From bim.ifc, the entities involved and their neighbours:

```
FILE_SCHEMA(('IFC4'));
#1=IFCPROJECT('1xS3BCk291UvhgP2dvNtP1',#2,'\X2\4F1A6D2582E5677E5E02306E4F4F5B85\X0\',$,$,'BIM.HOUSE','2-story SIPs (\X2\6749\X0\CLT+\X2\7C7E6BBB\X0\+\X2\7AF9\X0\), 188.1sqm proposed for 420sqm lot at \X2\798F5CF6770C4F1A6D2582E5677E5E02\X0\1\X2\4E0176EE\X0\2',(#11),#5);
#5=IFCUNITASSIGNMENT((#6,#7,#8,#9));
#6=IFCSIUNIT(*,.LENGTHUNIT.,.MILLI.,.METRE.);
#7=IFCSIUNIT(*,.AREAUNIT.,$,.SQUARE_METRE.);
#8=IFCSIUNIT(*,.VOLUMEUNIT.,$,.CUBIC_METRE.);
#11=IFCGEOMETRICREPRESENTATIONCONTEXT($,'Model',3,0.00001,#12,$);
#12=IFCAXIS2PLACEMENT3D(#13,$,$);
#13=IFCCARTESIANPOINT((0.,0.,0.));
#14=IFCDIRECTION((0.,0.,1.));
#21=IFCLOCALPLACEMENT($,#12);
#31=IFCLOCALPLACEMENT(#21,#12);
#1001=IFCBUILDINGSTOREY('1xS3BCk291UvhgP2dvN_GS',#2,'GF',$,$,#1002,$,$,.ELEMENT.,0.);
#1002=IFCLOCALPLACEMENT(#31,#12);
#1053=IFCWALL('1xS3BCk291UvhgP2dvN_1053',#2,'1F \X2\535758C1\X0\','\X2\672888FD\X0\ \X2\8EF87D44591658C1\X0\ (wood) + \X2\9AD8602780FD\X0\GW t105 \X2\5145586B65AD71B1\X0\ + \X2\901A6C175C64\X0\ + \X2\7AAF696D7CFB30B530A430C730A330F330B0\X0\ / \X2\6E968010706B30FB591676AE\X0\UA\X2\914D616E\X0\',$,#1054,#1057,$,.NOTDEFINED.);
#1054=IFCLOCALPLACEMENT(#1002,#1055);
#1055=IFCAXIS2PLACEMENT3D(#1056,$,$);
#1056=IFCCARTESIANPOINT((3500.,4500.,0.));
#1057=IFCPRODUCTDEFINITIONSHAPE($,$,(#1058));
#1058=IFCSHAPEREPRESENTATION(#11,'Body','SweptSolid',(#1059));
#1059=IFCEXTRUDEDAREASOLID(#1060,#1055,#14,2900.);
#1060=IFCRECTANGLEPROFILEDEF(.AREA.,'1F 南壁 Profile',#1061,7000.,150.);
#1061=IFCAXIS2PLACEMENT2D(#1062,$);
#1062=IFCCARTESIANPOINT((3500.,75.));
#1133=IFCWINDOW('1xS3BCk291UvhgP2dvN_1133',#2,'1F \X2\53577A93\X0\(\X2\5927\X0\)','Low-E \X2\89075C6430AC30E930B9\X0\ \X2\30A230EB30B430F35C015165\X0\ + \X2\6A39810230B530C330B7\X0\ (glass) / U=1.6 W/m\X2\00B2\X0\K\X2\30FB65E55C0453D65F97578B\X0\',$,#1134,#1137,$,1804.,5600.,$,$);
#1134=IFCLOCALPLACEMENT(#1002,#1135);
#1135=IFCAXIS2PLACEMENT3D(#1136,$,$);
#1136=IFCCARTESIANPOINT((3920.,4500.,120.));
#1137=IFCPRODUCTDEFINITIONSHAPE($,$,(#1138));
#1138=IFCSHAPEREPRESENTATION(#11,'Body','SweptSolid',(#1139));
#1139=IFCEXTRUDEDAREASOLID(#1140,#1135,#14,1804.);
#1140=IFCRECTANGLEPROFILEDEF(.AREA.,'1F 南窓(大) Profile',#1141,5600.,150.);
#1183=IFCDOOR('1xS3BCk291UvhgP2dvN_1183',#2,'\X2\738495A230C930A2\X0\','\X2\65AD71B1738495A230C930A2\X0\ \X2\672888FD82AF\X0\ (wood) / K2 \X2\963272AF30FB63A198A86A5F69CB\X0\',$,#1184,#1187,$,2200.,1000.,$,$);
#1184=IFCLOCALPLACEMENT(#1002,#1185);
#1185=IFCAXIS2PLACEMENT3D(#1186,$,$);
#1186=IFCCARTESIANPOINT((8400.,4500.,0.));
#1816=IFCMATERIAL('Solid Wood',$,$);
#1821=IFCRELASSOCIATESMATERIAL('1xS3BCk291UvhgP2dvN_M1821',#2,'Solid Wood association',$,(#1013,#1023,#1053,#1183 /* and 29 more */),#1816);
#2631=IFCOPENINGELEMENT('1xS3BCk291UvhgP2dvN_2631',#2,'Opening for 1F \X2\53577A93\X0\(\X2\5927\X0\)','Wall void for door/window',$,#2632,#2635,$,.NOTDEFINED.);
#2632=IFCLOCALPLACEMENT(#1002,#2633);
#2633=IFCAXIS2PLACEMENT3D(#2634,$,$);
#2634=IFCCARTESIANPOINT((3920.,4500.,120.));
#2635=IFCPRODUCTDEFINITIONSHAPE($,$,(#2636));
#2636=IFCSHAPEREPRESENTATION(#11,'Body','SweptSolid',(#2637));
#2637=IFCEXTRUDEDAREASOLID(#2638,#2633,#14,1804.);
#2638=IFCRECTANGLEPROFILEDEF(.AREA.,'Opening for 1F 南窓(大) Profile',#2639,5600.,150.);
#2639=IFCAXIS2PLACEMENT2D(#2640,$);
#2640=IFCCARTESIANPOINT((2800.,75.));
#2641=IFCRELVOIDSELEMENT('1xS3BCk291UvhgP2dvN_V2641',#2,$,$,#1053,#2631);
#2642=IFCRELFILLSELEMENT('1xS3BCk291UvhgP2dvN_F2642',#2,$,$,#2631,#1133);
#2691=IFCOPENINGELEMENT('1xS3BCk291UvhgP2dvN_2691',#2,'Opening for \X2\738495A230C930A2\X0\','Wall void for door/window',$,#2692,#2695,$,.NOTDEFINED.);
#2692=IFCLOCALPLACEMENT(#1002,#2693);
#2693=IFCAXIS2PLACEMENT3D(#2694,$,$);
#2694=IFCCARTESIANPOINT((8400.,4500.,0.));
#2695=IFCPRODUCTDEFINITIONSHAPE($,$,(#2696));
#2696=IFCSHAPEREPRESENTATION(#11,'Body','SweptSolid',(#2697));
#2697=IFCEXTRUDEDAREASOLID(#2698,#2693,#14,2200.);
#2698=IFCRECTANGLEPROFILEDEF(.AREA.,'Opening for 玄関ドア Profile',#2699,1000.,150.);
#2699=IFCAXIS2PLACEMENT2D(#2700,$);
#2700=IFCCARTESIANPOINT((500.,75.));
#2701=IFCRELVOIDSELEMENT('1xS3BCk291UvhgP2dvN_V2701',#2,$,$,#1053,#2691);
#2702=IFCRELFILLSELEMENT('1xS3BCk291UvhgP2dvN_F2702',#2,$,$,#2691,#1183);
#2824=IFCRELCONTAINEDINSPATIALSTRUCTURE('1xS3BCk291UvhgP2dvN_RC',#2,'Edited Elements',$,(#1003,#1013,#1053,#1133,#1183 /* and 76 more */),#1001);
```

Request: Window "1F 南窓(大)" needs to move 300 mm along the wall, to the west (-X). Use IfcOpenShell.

```python
import ifcopenshell
import ifcopenshell.api.geometry
import ifcopenshell.util.placement

model = ifcopenshell.open("bim.ifc")

window = model.by_guid("1xS3BCk291UvhgP2dvN_1133")
opening = window.FillsVoids[0].RelatingOpeningElement
wall = opening.VoidsElements[0].RelatingBuildingElement

wall_matrix = ifcopenshell.util.placement.get_local_placement(wall.ObjectPlacement)
shift = wall_matrix[:3, 0] * -300.0
before = ifcopenshell.util.placement.get_local_placement(window.ObjectPlacement)[:3, 3].copy()

# The window is not placed relative to its opening, so move both.
for product in (opening, window):
    matrix = ifcopenshell.util.placement.get_local_placement(product.ObjectPlacement)
    matrix[:3, 3] += shift
    ifcopenshell.api.geometry.edit_object_placement(model, product=product, matrix=matrix, is_si=False)

after = ifcopenshell.util.placement.get_local_placement(window.ObjectPlacement)[:3, 3]
print("window moved by", (after - before).round(3) + 0.0)

model.write("bim_edited.ifc")
```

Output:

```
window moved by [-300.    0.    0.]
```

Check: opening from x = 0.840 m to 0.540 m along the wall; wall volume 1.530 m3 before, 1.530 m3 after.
